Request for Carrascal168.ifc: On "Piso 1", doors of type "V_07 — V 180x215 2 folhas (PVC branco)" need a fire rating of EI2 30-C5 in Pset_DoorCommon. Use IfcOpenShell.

First a look at what the model holds.

```python
import ifcopenshell
import ifcopenshell.util.element

model = ifcopenshell.open("Carrascal168.ifc")
print(model.schema)
storey = next(s for s in model.by_type("IfcBuildingStorey") if s.Name == "Piso 1")
doors = [e for e in ifcopenshell.util.element.get_decomposition(storey) if e.is_a("IfcDoor")]
seen = {}
for e in doors:
    element_type = ifcopenshell.util.element.get_type(e)
    key = (element_type.Name if element_type != e and element_type else None, ifcopenshell.util.element.get_pset(e, "Pset_DoorCommon", "FireRating"))
    seen[key] = seen.get(key, 0) + 1
for (name, value), count in sorted(seen.items(), key=str):
    print(count, "x", name, "|", value)
```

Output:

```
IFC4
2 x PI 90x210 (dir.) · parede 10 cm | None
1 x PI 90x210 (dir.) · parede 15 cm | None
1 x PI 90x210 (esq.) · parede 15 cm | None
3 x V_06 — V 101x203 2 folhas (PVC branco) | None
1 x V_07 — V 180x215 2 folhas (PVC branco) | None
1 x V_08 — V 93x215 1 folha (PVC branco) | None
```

```python
import ifcopenshell
import ifcopenshell.api.pset
import ifcopenshell.util.element

model = ifcopenshell.open("Carrascal168.ifc")

storey = next(s for s in model.by_type("IfcBuildingStorey") if s.Name == "Piso 1")
doors = [e for e in ifcopenshell.util.element.get_decomposition(storey) if e.is_a("IfcDoor")]

count = 0
for e in doors:
    element_type = ifcopenshell.util.element.get_type(e)
    if element_type in (None, e) or element_type.Name != "V_07 — V 180x215 2 folhas (PVC branco)":
        continue
    # add_pset returns the element's existing set when there is one.
    pset = ifcopenshell.api.pset.add_pset(model, product=e, name="Pset_DoorCommon")
    ifcopenshell.api.pset.edit_pset(model, pset=pset, properties={"FireRating": "EI2 30-C5"})
    count += 1

print(count, "doors updated")

model.write("Carrascal168-out.ifc")
```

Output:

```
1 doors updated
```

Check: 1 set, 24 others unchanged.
